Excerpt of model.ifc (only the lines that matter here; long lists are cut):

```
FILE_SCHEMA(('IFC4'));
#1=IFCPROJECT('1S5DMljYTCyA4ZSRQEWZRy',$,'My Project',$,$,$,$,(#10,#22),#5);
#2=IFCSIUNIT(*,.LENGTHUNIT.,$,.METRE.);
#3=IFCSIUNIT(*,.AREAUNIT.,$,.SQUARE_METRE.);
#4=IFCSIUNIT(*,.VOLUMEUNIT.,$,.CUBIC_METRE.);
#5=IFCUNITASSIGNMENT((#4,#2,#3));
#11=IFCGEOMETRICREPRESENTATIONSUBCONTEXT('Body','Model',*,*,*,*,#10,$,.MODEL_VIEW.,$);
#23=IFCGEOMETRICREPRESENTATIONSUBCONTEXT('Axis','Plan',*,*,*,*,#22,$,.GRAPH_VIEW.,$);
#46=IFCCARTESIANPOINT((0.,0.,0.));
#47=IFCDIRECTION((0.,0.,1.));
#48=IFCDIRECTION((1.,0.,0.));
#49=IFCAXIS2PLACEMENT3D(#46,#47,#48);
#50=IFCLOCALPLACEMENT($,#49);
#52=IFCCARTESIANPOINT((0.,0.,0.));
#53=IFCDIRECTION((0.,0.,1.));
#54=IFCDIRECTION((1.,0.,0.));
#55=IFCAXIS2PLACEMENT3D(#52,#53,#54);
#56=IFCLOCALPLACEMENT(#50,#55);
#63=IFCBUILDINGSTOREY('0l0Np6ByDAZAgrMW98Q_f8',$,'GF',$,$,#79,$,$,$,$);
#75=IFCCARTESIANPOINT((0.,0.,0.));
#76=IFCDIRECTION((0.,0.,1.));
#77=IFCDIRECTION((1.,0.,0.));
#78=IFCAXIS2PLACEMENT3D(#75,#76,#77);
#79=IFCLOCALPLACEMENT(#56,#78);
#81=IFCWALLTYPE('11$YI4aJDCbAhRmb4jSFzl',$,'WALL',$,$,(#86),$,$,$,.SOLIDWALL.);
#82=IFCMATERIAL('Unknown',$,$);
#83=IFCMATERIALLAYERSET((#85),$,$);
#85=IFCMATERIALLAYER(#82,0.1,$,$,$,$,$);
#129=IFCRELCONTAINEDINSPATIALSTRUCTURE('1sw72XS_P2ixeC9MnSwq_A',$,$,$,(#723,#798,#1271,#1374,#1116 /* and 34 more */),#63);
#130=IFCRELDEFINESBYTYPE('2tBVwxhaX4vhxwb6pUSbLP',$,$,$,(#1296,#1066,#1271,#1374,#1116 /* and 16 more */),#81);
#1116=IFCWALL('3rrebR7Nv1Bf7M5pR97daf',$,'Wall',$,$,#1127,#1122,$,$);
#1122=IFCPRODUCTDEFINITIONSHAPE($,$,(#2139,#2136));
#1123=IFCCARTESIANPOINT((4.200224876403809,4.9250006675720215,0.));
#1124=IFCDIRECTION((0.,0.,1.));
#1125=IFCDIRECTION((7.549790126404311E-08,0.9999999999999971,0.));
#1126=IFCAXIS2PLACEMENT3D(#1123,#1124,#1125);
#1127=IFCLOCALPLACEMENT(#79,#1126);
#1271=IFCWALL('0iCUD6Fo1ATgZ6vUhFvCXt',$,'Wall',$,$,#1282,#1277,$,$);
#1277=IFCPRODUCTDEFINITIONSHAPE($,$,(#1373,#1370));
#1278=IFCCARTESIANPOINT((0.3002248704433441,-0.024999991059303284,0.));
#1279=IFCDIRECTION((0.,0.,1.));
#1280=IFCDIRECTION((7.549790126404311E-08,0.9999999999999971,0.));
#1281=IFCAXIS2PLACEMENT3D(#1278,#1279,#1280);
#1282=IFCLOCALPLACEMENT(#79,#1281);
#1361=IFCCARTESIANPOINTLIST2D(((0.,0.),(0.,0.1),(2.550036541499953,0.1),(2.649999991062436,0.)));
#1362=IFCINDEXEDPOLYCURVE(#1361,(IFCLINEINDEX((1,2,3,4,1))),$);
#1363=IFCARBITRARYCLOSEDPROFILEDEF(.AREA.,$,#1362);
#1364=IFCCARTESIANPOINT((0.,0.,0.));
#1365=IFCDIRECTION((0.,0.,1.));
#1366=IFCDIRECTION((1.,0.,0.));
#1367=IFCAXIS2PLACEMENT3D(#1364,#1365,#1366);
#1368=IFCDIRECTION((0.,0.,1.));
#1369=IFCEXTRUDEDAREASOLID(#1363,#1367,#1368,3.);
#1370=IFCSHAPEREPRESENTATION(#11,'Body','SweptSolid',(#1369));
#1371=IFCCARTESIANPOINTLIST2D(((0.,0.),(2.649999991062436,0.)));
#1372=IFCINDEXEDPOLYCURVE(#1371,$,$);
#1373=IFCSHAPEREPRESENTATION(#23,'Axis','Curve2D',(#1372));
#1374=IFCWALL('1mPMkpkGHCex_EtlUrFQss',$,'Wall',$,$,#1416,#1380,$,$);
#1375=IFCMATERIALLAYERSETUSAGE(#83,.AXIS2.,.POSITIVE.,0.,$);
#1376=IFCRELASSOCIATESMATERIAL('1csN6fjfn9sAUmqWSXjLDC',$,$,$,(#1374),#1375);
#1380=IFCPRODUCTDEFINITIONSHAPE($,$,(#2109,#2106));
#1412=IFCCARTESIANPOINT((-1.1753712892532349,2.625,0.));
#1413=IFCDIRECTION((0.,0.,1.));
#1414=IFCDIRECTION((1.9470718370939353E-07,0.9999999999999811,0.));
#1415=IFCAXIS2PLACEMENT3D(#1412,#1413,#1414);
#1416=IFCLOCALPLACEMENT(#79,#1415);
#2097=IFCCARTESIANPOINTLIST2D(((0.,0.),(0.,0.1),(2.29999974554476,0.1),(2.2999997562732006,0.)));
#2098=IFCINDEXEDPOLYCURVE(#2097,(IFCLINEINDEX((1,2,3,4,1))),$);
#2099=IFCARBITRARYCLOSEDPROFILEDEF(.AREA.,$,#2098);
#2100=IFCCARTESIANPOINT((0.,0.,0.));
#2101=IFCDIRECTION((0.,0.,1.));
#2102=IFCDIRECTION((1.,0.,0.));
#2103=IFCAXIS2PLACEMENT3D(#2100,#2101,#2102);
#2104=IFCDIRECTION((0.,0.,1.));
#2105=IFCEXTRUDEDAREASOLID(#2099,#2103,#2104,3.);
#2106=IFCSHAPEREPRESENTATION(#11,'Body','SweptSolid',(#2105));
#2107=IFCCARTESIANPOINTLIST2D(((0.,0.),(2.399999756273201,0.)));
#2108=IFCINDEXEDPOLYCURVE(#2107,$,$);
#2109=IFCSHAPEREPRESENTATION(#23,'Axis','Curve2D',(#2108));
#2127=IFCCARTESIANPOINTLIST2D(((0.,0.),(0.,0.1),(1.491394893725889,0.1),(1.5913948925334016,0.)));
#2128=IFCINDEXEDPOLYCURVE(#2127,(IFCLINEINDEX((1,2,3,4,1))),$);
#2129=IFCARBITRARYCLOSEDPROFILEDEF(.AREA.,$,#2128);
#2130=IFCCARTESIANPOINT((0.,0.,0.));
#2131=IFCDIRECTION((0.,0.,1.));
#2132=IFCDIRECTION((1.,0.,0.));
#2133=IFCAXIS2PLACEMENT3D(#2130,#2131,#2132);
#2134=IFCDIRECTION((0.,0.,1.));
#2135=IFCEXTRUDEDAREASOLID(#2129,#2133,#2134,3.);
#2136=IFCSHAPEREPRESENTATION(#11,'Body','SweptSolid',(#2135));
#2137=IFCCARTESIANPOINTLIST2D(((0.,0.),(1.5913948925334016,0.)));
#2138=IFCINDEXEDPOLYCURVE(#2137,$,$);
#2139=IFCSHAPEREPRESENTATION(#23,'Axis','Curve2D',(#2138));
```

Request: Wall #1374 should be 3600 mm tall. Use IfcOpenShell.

```python
import ifcopenshell
import ifcopenshell.geom
import ifcopenshell.util.representation
import ifcopenshell.util.shape
import ifcopenshell.util.unit

model = ifcopenshell.open("model.ifc")
unit_scale = ifcopenshell.util.unit.calculate_unit_scale(model)
settings = ifcopenshell.geom.settings()


def volume(element):
    """Net volume in cubic metres, openings subtracted."""
    shape = ifcopenshell.geom.create_shape(settings, element)
    return ifcopenshell.util.shape.get_volume(shape.geometry)


wall = model.by_guid("1mPMkpkGHCex_EtlUrFQss")
before = volume(wall)

body = ifcopenshell.util.representation.get_representation(wall, "Model", "Body")
solid = body.Items[0]
old_height = solid.Depth
solid.Depth = 3.6 / unit_scale
after = volume(wall)

print(f"height {old_height:g} -> {solid.Depth:g}, volume {before:.3f} -> {after:.3f} m3")

model.write("model_edited.ifc")
```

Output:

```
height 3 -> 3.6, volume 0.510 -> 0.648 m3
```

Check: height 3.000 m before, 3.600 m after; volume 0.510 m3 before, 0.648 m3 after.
